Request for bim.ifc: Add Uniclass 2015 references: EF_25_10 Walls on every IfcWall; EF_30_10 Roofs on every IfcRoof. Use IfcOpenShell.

First a look at what the model holds.

```python
import ifcopenshell

model = ifcopenshell.open("bim.ifc")
print(model.schema)
print("classifications:", [c.Name for c in model.by_type("IfcClassification")])
for ifc_class in ("IfcDoor", "IfcRoof", "IfcStair", "IfcWall", "IfcWindow"):
    print(ifc_class, len(model.by_type(ifc_class)))
```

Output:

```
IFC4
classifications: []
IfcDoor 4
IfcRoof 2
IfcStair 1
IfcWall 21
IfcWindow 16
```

```python
import ifcopenshell
import ifcopenshell.api.classification

model = ifcopenshell.open("bim.ifc")

system = ifcopenshell.api.classification.add_classification(model, classification="Uniclass 2015")

codes = {
    "IfcWall": ("EF_25_10", "Walls"),
    "IfcRoof": ("EF_30_10", "Roofs"),
}
for ifc_class, (code, name) in codes.items():
    products = model.by_type(ifc_class)
    ifcopenshell.api.classification.add_reference(
        model, products=products, classification=system, identification=code, name=name
    )
    print(code, len(products))

model.write("bim-out.ifc")
```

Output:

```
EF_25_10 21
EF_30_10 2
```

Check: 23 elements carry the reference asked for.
